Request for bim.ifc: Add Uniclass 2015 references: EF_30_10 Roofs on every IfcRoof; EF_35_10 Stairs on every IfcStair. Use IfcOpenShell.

First a look at what the model holds.

```python
import ifcopenshell

model = ifcopenshell.open("bim.ifc")
print(model.schema)
print("classifications:", [c.Name for c in model.by_type("IfcClassification")])
for ifc_class in ("IfcDoor", "IfcRoof", "IfcStair", "IfcWall", "IfcWindow"):
    print(ifc_class, len(model.by_type(ifc_class)))
```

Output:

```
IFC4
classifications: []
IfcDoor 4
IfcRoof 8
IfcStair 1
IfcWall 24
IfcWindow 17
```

```python
import ifcopenshell
import ifcopenshell.api.classification

model = ifcopenshell.open("bim.ifc")

system = ifcopenshell.api.classification.add_classification(model, classification="Uniclass 2015")

codes = {
    "IfcRoof": ("EF_30_10", "Roofs"),
    "IfcStair": ("EF_35_10", "Stairs"),
}
for ifc_class, (code, name) in codes.items():
    products = model.by_type(ifc_class)
    ifcopenshell.api.classification.add_reference(
        model, products=products, classification=system, identification=code, name=name
    )
    print(code, len(products))

model.write("bim_rev.ifc")
```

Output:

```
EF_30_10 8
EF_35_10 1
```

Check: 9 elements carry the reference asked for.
